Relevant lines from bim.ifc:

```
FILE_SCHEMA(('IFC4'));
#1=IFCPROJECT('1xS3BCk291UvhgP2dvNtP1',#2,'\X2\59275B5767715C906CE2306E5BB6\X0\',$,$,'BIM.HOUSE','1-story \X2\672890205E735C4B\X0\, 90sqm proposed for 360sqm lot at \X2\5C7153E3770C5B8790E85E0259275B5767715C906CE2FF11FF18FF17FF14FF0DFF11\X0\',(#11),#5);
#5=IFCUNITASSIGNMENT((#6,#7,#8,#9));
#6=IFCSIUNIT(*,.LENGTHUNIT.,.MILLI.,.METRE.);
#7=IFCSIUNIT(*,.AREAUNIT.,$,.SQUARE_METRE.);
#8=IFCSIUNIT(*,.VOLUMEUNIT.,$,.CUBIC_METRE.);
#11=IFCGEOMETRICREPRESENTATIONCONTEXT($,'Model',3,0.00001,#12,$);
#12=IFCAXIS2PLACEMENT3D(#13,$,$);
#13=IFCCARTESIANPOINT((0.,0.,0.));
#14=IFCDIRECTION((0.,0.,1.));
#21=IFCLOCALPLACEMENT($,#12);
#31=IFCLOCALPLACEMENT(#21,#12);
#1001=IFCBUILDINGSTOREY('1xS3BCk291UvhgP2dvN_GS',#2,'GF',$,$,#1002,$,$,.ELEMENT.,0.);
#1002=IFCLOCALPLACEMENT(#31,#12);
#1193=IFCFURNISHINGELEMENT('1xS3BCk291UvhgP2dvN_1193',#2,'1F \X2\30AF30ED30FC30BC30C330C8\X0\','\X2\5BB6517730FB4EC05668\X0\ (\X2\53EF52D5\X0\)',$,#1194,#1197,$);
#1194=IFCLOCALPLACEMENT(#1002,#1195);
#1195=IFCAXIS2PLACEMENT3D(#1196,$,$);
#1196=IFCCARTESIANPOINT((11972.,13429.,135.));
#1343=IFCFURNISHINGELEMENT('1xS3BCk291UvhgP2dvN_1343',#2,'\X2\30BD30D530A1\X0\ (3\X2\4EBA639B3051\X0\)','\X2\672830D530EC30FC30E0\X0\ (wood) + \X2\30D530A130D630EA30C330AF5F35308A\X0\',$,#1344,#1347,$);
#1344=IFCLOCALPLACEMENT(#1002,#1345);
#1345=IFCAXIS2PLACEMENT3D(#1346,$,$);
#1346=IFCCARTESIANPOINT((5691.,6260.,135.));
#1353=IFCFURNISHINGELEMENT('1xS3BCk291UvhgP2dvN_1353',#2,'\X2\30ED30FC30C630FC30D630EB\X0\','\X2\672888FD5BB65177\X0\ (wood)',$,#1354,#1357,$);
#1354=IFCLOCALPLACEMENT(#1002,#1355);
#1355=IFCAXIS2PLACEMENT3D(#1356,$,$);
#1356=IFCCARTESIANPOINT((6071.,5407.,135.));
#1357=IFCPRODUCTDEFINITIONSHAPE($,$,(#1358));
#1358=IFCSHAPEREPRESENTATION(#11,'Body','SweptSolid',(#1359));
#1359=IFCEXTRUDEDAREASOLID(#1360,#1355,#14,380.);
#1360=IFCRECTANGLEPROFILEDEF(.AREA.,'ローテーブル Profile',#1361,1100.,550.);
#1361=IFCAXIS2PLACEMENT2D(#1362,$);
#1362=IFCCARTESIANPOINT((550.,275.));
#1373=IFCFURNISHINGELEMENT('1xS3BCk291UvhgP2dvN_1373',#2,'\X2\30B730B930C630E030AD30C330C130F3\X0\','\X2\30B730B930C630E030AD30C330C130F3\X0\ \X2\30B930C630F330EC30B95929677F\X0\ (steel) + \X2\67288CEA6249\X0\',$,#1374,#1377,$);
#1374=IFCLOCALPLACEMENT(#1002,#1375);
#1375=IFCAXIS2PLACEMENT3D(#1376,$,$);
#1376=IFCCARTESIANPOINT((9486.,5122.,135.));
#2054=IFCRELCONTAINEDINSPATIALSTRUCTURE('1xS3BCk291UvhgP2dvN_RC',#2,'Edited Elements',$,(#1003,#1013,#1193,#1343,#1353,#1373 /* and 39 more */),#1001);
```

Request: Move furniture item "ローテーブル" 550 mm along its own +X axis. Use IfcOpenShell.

```python
import ifcopenshell
import ifcopenshell.api.geometry
import ifcopenshell.util.placement
import ifcopenshell.util.unit

model = ifcopenshell.open("bim.ifc")
unit_scale = ifcopenshell.util.unit.calculate_unit_scale(model)

item = model.by_id(1353)
matrix = ifcopenshell.util.placement.get_local_placement(item.ObjectPlacement)
matrix[:3, 3] += matrix[:3, 0] * 0.55 / unit_scale
ifcopenshell.api.geometry.edit_object_placement(model, product=item, matrix=matrix, is_si=False)

print(ifcopenshell.util.placement.get_local_placement(item.ObjectPlacement).round(3) + 0.0)

model.write("bim_rev.ifc")
```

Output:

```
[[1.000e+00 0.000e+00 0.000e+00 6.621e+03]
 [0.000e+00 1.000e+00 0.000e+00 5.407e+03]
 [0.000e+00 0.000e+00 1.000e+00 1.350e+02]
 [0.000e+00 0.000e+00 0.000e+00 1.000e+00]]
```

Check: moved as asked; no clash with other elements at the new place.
